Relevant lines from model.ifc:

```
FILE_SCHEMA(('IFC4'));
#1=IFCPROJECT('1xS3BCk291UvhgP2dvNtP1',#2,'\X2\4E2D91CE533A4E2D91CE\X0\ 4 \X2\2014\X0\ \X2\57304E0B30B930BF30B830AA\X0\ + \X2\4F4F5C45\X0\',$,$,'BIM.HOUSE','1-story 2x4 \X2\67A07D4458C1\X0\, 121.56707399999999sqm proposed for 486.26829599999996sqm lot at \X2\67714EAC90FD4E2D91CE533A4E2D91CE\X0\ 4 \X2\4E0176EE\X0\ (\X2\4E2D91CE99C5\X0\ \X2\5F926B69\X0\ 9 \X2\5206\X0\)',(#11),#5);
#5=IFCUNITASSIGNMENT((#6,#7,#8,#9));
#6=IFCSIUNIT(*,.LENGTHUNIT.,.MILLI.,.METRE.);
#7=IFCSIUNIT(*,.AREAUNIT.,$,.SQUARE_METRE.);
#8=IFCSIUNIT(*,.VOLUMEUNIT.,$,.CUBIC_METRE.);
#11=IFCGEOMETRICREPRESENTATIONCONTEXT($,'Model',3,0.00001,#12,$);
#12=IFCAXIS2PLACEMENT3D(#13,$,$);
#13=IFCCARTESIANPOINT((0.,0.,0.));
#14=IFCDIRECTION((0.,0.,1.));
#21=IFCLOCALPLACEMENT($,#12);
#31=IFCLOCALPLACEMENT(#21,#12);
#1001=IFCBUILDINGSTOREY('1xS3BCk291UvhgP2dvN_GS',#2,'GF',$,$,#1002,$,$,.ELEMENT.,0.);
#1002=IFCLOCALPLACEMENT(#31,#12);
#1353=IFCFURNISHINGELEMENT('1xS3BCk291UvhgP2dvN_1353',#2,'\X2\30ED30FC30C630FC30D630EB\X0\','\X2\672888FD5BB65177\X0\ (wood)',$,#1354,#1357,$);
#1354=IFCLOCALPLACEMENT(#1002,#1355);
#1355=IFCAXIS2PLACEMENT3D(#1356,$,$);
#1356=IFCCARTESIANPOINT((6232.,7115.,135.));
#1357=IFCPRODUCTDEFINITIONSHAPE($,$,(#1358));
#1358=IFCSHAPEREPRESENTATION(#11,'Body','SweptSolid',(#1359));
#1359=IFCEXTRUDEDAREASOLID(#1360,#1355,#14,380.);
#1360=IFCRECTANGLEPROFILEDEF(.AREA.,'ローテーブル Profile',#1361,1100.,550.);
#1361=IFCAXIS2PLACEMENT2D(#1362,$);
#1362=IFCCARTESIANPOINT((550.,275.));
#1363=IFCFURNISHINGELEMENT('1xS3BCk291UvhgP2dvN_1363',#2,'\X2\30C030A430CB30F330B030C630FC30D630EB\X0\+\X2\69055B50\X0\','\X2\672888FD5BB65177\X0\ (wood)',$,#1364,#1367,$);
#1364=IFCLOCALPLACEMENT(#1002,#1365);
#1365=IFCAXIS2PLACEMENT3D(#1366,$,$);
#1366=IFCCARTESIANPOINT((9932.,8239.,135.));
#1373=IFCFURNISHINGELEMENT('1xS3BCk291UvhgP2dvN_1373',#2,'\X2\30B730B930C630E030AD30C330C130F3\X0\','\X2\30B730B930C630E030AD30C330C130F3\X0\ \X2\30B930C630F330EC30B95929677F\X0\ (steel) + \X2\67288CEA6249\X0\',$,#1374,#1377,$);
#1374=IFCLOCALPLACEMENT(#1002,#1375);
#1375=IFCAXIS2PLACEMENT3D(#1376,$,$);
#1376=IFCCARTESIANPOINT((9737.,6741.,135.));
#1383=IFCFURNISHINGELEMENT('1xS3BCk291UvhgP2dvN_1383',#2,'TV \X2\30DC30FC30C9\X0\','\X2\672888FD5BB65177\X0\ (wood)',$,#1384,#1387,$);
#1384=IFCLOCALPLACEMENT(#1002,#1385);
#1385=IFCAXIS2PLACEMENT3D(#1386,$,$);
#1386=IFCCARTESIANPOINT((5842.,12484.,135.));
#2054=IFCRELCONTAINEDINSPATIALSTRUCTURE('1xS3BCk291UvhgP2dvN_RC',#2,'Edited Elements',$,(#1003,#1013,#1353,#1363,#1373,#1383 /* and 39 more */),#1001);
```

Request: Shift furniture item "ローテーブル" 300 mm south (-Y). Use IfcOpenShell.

```python
import ifcopenshell
import ifcopenshell.api.geometry
import ifcopenshell.util.placement

model = ifcopenshell.open("model.ifc")

item = model.by_guid("1xS3BCk291UvhgP2dvN_1353")
matrix = ifcopenshell.util.placement.get_local_placement(item.ObjectPlacement)
matrix[1, 3] -= 300.0
ifcopenshell.api.geometry.edit_object_placement(model, product=item, matrix=matrix, is_si=False)

print(ifcopenshell.util.placement.get_local_placement(item.ObjectPlacement).round(3) + 0.0)

model.write("model_v2.ifc")
```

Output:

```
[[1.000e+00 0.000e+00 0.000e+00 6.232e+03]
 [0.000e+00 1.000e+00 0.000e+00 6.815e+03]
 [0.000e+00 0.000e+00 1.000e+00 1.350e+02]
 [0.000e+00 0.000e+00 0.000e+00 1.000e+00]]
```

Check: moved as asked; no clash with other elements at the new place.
